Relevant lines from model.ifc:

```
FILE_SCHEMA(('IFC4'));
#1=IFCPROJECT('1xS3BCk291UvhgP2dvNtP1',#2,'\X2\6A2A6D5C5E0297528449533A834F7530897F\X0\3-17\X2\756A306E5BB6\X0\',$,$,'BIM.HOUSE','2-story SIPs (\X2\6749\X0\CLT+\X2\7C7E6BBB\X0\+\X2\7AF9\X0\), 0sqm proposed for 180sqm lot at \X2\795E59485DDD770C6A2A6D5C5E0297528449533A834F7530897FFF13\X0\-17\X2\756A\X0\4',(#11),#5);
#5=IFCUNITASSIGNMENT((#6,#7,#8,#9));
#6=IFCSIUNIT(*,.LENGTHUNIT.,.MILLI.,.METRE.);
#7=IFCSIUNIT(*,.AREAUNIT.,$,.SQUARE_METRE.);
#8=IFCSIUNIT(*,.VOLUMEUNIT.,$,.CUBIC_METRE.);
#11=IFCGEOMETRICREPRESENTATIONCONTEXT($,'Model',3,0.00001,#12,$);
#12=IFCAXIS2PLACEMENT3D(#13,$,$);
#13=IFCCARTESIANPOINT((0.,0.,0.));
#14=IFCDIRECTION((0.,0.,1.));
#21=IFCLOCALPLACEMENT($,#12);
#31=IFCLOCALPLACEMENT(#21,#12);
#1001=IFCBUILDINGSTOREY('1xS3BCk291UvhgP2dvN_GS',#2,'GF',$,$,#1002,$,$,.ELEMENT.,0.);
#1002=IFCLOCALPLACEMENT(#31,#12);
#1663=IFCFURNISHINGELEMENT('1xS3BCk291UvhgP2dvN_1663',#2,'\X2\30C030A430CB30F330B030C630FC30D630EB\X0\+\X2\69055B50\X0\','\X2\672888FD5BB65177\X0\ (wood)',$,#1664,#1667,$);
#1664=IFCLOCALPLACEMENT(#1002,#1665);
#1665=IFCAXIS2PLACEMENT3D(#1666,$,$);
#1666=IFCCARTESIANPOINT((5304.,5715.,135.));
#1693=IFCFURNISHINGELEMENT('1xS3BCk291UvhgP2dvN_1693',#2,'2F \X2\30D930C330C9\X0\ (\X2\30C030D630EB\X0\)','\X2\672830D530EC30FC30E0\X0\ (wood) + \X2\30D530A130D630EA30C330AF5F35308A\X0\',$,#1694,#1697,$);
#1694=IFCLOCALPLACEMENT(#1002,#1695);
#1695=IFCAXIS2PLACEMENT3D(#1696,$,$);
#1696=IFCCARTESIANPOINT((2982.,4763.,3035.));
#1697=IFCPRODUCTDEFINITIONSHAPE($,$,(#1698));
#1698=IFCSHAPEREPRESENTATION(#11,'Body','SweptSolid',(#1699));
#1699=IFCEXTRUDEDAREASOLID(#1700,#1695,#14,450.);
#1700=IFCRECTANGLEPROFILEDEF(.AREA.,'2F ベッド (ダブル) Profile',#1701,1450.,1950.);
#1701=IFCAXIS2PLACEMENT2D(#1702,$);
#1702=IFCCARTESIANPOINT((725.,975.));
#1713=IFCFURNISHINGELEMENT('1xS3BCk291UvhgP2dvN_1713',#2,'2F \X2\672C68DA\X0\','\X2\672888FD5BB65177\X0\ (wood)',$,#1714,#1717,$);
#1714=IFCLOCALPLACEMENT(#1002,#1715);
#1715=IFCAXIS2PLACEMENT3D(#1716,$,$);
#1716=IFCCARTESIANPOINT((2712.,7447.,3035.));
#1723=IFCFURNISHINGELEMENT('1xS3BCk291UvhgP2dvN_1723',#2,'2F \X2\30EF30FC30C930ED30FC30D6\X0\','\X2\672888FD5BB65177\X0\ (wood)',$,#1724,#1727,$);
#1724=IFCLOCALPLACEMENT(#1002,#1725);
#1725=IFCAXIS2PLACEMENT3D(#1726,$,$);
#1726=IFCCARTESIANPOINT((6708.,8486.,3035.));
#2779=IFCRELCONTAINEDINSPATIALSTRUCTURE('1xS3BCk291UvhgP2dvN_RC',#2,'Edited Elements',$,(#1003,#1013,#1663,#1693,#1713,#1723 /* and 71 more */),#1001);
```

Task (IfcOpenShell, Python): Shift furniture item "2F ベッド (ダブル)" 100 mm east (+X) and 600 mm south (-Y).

```python
import ifcopenshell
import ifcopenshell.api.geometry
import ifcopenshell.util.placement
import ifcopenshell.util.unit

model = ifcopenshell.open("model.ifc")
unit_scale = ifcopenshell.util.unit.calculate_unit_scale(model)

item = model.by_guid("1xS3BCk291UvhgP2dvN_1693")
matrix = ifcopenshell.util.placement.get_local_placement(item.ObjectPlacement)
matrix[0, 3] += 0.1 / unit_scale
matrix[1, 3] -= 0.6 / unit_scale
ifcopenshell.api.geometry.edit_object_placement(model, product=item, matrix=matrix, is_si=False)

print(ifcopenshell.util.placement.get_local_placement(item.ObjectPlacement).round(3) + 0.0)

model.write("model-out.ifc")
```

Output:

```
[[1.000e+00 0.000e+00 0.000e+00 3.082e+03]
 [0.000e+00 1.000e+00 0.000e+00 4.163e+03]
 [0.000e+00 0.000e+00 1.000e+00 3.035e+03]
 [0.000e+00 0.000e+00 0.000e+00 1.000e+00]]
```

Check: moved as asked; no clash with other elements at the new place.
